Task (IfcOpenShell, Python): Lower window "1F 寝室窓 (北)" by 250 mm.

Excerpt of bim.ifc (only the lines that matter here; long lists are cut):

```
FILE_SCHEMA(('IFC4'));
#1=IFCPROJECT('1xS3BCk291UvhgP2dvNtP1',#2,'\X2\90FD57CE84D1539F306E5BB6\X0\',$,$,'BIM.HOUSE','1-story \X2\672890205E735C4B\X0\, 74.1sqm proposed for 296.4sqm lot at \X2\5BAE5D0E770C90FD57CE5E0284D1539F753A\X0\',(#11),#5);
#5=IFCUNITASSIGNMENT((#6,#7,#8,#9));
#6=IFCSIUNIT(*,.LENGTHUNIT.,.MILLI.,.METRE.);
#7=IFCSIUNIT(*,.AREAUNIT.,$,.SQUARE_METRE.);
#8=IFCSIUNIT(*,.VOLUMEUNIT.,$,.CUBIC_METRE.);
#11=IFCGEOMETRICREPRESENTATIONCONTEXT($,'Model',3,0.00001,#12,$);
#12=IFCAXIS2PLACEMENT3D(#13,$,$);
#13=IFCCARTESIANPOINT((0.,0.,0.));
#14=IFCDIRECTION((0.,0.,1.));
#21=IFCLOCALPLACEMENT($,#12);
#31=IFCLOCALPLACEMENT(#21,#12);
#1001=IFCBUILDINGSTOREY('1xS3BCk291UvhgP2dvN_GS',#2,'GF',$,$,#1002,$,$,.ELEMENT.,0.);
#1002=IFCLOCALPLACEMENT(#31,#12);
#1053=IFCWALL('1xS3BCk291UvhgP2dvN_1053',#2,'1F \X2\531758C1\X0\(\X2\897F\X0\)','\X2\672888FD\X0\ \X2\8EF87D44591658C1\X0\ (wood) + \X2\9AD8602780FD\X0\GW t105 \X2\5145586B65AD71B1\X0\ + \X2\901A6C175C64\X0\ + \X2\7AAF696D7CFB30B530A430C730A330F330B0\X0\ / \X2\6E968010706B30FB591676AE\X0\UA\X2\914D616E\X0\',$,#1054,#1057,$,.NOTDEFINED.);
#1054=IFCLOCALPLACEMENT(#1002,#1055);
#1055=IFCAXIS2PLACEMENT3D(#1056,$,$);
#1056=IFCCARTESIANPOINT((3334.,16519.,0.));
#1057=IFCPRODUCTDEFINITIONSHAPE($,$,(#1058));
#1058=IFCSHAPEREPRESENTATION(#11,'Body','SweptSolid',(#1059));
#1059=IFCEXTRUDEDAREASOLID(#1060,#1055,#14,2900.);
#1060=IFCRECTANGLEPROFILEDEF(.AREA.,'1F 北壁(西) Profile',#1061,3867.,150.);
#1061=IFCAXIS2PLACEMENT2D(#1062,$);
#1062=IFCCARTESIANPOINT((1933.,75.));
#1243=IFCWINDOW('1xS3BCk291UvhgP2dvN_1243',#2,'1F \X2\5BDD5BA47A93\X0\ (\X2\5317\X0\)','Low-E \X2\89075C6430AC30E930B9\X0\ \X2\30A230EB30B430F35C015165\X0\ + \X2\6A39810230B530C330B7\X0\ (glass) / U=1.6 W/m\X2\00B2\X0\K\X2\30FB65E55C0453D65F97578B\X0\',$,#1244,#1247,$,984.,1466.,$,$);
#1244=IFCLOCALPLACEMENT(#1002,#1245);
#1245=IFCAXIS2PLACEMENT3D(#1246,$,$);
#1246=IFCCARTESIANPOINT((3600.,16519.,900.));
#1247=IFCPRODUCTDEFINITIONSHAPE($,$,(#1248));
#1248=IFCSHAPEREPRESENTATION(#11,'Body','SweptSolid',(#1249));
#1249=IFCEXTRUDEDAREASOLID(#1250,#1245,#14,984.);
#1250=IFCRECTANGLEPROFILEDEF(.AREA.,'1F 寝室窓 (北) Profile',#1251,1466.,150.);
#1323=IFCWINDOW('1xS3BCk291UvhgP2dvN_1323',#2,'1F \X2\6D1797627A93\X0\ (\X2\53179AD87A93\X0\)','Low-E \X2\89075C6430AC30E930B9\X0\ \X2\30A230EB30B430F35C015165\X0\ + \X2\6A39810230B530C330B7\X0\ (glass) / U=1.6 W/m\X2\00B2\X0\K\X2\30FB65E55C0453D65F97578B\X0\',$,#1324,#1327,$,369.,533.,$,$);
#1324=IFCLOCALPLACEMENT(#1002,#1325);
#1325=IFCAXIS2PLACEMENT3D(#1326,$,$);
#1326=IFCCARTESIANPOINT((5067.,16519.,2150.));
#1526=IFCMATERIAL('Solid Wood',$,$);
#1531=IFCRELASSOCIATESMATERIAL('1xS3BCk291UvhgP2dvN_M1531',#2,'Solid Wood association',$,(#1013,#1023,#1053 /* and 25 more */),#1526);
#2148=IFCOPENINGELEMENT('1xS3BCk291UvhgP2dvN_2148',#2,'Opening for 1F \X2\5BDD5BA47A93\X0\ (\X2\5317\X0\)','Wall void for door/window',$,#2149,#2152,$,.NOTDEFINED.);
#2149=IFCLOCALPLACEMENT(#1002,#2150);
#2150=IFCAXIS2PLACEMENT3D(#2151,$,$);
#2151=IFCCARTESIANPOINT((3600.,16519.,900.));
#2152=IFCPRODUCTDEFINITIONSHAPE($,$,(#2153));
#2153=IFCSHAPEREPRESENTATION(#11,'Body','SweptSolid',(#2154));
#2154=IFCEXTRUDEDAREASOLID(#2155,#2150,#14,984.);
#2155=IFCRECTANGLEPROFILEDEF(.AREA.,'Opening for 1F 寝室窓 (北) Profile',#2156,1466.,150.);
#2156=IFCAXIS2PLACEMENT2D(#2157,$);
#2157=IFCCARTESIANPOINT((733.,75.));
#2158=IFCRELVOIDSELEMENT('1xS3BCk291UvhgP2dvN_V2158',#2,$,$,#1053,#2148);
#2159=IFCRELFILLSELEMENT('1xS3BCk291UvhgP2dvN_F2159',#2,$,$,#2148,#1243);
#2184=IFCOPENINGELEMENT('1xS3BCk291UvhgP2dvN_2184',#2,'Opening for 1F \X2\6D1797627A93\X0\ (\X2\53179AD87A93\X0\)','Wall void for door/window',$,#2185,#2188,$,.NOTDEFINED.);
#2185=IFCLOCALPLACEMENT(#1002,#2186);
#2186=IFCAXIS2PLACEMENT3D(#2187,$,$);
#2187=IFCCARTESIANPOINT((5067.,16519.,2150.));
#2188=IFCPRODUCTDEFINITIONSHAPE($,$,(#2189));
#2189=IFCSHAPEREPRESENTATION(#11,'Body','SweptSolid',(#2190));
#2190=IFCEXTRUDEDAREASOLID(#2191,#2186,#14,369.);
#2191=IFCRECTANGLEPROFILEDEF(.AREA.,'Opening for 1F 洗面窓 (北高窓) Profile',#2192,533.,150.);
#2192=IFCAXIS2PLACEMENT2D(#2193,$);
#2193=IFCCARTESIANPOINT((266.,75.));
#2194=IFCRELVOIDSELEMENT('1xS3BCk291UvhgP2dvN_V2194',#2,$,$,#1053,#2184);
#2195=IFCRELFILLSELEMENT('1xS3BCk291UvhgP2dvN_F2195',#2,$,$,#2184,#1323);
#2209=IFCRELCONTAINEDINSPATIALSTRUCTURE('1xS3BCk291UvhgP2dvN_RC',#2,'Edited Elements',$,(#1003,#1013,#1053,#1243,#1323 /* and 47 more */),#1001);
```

```python
import numpy as np
import ifcopenshell
import ifcopenshell.api.geometry
import ifcopenshell.util.placement
import ifcopenshell.util.unit

model = ifcopenshell.open("bim.ifc")
unit_scale = ifcopenshell.util.unit.calculate_unit_scale(model)

window = model.by_guid("1xS3BCk291UvhgP2dvN_1243")
opening = window.FillsVoids[0].RelatingOpeningElement
dz = -0.25 / unit_scale

shift = np.array([0.0, 0.0, dz])
# The window is not placed relative to its opening, so move both.
for product in (opening, window):
    matrix = ifcopenshell.util.placement.get_local_placement(product.ObjectPlacement)
    matrix[:3, 3] += shift
    ifcopenshell.api.geometry.edit_object_placement(model, product=product, matrix=matrix, is_si=False)

print(f"moved by {dz * unit_scale:+.3f} m")

model.write("bim-out.ifc")
```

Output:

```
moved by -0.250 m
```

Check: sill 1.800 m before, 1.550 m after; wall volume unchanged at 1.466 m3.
